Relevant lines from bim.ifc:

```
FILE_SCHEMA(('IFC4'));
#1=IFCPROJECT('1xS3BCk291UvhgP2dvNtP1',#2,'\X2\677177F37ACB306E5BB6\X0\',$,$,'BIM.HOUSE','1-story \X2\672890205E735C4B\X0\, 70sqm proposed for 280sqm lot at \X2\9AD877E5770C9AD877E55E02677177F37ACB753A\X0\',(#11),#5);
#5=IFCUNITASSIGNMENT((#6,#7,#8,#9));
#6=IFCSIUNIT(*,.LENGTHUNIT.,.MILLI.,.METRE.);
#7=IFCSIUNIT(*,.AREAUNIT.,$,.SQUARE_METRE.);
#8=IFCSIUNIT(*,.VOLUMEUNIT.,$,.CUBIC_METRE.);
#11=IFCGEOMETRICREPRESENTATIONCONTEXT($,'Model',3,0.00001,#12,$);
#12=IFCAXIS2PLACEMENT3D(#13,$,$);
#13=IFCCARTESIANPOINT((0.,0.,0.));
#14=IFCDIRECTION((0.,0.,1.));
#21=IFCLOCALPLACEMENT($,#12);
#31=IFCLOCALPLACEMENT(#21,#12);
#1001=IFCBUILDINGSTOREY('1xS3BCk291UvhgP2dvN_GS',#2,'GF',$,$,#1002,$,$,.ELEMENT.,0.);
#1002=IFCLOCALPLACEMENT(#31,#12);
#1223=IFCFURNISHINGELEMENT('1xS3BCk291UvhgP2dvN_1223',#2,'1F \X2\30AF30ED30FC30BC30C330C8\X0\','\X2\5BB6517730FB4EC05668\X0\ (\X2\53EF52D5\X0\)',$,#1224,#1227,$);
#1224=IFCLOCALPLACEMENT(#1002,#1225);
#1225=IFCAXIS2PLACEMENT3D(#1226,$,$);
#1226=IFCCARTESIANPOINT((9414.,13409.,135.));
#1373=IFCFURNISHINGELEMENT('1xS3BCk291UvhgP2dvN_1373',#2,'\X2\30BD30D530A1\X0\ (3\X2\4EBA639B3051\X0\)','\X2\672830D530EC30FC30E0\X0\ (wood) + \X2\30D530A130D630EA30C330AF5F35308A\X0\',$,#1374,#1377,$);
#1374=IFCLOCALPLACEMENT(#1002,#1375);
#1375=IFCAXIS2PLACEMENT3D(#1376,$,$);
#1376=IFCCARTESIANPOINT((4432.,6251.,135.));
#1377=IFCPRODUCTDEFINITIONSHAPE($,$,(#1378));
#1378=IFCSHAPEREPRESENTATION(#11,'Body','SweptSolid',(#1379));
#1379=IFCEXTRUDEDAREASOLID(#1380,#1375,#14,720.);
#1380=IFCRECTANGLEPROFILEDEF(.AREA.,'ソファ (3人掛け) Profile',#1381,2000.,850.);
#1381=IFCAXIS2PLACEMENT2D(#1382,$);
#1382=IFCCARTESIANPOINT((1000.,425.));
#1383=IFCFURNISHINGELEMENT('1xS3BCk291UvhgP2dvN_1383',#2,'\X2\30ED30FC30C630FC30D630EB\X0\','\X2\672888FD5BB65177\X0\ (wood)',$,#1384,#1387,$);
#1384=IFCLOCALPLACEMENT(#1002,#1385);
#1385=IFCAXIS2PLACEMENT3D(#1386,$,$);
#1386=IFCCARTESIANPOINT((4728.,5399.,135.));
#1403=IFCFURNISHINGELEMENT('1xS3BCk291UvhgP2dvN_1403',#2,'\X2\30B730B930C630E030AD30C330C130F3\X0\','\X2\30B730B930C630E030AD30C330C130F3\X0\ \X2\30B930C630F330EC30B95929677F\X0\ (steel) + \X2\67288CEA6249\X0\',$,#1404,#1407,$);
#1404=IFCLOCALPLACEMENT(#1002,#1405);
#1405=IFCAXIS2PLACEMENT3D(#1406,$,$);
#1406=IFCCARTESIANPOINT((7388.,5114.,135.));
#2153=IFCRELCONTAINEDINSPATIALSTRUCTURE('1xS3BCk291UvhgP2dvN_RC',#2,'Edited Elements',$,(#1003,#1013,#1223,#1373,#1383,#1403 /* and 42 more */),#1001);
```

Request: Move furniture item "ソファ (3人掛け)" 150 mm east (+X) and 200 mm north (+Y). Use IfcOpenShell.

```python
import ifcopenshell
import ifcopenshell.api.geometry
import ifcopenshell.util.placement
import ifcopenshell.util.unit

model = ifcopenshell.open("bim.ifc")
unit_scale = ifcopenshell.util.unit.calculate_unit_scale(model)

item = model.by_guid("1xS3BCk291UvhgP2dvN_1373")
matrix = ifcopenshell.util.placement.get_local_placement(item.ObjectPlacement)
matrix[0, 3] += 0.15 / unit_scale
matrix[1, 3] += 0.2 / unit_scale
ifcopenshell.api.geometry.edit_object_placement(model, product=item, matrix=matrix, is_si=False)

print(ifcopenshell.util.placement.get_local_placement(item.ObjectPlacement).round(3) + 0.0)

model.write("bim_rev.ifc")
```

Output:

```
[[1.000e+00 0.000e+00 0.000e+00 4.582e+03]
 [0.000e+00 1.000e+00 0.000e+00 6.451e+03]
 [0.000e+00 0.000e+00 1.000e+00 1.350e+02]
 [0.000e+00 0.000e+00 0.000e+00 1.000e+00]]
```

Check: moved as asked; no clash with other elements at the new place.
